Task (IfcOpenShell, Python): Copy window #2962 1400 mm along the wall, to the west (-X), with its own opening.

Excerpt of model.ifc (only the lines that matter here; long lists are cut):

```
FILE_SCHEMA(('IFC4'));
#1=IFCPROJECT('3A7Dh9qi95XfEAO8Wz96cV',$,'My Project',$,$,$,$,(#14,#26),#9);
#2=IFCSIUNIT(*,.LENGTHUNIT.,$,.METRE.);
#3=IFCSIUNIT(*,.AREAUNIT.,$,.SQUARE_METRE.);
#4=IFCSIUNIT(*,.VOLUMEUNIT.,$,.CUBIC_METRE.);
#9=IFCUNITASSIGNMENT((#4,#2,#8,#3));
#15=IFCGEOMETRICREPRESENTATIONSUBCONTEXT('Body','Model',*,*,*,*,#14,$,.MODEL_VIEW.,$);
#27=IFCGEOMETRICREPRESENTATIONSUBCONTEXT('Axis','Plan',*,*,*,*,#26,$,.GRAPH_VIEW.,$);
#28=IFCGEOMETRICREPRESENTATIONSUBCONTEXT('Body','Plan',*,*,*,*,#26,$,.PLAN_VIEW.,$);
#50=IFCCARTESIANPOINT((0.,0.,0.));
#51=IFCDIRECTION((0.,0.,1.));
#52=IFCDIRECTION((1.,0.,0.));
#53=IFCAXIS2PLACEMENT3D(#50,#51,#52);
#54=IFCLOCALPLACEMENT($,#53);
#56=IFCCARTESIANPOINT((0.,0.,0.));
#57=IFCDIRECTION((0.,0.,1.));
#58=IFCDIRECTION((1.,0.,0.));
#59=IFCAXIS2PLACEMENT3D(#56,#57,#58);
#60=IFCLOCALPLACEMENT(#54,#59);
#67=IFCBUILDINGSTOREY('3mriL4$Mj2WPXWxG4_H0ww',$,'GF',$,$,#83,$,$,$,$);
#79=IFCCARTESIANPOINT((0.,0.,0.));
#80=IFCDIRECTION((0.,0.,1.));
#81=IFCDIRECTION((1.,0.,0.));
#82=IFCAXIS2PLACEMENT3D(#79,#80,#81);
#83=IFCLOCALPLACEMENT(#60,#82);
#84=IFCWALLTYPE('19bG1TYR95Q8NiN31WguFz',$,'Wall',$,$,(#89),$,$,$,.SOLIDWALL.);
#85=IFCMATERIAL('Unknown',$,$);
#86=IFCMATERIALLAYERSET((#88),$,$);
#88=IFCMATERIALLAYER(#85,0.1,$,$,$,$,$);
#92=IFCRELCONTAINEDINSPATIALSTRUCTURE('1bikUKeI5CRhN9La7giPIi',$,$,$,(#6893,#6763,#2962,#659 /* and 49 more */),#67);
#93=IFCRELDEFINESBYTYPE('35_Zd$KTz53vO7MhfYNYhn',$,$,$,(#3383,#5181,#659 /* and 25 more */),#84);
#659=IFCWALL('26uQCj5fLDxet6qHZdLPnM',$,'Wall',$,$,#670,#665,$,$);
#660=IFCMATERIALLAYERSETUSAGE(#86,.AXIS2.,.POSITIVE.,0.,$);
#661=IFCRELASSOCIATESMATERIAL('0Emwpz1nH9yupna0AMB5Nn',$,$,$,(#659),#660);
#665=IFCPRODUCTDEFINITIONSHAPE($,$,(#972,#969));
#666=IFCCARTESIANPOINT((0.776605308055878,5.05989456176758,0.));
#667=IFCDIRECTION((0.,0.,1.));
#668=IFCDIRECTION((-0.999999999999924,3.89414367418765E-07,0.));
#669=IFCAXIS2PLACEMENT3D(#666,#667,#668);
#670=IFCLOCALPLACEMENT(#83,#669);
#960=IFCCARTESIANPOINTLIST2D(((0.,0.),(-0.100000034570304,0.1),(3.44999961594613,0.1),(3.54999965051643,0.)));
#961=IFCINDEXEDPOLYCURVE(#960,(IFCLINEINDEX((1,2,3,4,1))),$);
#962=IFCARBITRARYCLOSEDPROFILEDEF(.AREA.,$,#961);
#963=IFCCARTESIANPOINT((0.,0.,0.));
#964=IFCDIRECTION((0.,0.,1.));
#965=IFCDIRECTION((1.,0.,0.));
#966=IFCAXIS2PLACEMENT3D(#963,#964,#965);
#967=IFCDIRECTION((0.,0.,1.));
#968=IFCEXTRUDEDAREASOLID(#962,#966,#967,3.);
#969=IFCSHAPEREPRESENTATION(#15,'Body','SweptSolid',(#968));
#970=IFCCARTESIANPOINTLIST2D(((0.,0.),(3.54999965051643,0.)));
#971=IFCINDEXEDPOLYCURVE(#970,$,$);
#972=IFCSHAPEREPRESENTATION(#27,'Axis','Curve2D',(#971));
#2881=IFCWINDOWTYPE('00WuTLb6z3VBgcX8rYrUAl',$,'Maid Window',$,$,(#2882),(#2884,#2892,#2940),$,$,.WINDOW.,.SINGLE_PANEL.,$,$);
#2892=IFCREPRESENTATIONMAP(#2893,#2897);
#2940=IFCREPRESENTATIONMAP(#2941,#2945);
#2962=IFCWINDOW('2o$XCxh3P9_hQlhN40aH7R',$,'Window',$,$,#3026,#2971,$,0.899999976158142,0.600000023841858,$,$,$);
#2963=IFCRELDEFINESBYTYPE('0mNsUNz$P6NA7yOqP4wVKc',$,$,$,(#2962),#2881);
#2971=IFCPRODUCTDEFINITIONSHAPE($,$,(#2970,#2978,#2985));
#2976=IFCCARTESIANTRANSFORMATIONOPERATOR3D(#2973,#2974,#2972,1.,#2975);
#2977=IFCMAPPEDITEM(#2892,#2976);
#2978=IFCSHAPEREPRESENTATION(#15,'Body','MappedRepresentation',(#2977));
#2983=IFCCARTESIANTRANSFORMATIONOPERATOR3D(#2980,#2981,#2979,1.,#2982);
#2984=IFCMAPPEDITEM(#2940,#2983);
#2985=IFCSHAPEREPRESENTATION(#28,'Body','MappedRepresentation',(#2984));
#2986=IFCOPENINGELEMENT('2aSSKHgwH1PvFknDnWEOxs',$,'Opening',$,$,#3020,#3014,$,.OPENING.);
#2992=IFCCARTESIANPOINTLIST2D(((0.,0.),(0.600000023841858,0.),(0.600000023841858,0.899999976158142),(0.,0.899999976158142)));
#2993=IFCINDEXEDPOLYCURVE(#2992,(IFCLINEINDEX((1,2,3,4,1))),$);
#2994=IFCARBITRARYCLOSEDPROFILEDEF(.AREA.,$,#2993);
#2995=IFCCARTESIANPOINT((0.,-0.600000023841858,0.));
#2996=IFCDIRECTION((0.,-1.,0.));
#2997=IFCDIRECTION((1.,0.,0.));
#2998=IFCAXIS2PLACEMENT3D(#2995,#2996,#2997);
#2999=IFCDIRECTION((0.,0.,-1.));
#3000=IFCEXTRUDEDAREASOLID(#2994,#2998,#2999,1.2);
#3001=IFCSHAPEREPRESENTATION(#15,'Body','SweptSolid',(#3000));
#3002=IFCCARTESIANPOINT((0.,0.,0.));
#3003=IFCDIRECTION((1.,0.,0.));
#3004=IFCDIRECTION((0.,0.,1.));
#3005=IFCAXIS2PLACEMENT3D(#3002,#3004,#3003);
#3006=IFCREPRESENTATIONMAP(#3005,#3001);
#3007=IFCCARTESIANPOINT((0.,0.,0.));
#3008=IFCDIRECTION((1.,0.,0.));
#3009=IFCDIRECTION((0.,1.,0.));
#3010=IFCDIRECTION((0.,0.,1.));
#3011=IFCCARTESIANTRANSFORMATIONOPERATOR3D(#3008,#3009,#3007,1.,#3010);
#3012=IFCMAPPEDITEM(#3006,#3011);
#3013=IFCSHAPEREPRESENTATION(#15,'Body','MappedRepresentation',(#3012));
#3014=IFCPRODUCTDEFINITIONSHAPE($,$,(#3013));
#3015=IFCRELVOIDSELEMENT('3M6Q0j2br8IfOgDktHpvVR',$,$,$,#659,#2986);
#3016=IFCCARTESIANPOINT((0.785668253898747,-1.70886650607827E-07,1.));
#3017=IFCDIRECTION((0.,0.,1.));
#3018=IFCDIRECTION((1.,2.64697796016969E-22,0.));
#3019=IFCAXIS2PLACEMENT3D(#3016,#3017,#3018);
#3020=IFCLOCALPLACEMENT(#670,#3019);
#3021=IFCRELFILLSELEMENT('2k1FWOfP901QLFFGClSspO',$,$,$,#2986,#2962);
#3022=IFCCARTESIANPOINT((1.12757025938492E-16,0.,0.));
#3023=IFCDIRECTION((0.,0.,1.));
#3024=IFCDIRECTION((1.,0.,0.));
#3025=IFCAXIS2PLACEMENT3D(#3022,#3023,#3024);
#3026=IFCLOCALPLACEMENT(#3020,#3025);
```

```python
import ifcopenshell
import ifcopenshell.api.feature
import ifcopenshell.api.geometry
import ifcopenshell.api.root
import ifcopenshell.geom
import ifcopenshell.util.element
import ifcopenshell.util.placement
import ifcopenshell.util.shape

model = ifcopenshell.open("model.ifc")
settings = ifcopenshell.geom.settings()


def volume(element):
    """Net volume in cubic metres, openings subtracted."""
    shape = ifcopenshell.geom.create_shape(settings, element)
    return ifcopenshell.util.shape.get_volume(shape.geometry)


window = model.by_guid("2o$XCxh3P9_hQlhN40aH7R")
opening = window.FillsVoids[0].RelatingOpeningElement
wall = opening.VoidsElements[0].RelatingBuildingElement
before = volume(wall)
shift = ifcopenshell.util.placement.get_local_placement(wall.ObjectPlacement)[:3, 0] * 1.4

# copy_class copies the void relationship, type, container and properties, but no geometry.
new_opening = ifcopenshell.api.root.copy_class(model, product=opening)
new_opening.Representation = ifcopenshell.util.element.copy_deep(
    model, opening.Representation, exclude=["IfcGeometricRepresentationContext", "IfcRepresentationMap"]
)
new_window = ifcopenshell.api.root.copy_class(model, product=window)
new_window.Representation = ifcopenshell.util.element.copy_deep(
    model, window.Representation, exclude=["IfcGeometricRepresentationContext", "IfcRepresentationMap"]
)
ifcopenshell.api.feature.add_filling(model, opening=new_opening, element=new_window)

for old, new in ((opening, new_opening), (window, new_window)):
    matrix = ifcopenshell.util.placement.get_local_placement(old.ObjectPlacement)
    matrix[:3, 3] += shift
    ifcopenshell.api.geometry.edit_object_placement(model, product=new, matrix=matrix, is_si=False)

after = volume(wall)

print(f"wall volume {before:.3f} -> {after:.3f} m3")

model.write("model_v2.ifc")
```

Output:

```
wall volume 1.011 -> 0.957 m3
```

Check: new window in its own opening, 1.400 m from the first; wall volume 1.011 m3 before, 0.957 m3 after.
